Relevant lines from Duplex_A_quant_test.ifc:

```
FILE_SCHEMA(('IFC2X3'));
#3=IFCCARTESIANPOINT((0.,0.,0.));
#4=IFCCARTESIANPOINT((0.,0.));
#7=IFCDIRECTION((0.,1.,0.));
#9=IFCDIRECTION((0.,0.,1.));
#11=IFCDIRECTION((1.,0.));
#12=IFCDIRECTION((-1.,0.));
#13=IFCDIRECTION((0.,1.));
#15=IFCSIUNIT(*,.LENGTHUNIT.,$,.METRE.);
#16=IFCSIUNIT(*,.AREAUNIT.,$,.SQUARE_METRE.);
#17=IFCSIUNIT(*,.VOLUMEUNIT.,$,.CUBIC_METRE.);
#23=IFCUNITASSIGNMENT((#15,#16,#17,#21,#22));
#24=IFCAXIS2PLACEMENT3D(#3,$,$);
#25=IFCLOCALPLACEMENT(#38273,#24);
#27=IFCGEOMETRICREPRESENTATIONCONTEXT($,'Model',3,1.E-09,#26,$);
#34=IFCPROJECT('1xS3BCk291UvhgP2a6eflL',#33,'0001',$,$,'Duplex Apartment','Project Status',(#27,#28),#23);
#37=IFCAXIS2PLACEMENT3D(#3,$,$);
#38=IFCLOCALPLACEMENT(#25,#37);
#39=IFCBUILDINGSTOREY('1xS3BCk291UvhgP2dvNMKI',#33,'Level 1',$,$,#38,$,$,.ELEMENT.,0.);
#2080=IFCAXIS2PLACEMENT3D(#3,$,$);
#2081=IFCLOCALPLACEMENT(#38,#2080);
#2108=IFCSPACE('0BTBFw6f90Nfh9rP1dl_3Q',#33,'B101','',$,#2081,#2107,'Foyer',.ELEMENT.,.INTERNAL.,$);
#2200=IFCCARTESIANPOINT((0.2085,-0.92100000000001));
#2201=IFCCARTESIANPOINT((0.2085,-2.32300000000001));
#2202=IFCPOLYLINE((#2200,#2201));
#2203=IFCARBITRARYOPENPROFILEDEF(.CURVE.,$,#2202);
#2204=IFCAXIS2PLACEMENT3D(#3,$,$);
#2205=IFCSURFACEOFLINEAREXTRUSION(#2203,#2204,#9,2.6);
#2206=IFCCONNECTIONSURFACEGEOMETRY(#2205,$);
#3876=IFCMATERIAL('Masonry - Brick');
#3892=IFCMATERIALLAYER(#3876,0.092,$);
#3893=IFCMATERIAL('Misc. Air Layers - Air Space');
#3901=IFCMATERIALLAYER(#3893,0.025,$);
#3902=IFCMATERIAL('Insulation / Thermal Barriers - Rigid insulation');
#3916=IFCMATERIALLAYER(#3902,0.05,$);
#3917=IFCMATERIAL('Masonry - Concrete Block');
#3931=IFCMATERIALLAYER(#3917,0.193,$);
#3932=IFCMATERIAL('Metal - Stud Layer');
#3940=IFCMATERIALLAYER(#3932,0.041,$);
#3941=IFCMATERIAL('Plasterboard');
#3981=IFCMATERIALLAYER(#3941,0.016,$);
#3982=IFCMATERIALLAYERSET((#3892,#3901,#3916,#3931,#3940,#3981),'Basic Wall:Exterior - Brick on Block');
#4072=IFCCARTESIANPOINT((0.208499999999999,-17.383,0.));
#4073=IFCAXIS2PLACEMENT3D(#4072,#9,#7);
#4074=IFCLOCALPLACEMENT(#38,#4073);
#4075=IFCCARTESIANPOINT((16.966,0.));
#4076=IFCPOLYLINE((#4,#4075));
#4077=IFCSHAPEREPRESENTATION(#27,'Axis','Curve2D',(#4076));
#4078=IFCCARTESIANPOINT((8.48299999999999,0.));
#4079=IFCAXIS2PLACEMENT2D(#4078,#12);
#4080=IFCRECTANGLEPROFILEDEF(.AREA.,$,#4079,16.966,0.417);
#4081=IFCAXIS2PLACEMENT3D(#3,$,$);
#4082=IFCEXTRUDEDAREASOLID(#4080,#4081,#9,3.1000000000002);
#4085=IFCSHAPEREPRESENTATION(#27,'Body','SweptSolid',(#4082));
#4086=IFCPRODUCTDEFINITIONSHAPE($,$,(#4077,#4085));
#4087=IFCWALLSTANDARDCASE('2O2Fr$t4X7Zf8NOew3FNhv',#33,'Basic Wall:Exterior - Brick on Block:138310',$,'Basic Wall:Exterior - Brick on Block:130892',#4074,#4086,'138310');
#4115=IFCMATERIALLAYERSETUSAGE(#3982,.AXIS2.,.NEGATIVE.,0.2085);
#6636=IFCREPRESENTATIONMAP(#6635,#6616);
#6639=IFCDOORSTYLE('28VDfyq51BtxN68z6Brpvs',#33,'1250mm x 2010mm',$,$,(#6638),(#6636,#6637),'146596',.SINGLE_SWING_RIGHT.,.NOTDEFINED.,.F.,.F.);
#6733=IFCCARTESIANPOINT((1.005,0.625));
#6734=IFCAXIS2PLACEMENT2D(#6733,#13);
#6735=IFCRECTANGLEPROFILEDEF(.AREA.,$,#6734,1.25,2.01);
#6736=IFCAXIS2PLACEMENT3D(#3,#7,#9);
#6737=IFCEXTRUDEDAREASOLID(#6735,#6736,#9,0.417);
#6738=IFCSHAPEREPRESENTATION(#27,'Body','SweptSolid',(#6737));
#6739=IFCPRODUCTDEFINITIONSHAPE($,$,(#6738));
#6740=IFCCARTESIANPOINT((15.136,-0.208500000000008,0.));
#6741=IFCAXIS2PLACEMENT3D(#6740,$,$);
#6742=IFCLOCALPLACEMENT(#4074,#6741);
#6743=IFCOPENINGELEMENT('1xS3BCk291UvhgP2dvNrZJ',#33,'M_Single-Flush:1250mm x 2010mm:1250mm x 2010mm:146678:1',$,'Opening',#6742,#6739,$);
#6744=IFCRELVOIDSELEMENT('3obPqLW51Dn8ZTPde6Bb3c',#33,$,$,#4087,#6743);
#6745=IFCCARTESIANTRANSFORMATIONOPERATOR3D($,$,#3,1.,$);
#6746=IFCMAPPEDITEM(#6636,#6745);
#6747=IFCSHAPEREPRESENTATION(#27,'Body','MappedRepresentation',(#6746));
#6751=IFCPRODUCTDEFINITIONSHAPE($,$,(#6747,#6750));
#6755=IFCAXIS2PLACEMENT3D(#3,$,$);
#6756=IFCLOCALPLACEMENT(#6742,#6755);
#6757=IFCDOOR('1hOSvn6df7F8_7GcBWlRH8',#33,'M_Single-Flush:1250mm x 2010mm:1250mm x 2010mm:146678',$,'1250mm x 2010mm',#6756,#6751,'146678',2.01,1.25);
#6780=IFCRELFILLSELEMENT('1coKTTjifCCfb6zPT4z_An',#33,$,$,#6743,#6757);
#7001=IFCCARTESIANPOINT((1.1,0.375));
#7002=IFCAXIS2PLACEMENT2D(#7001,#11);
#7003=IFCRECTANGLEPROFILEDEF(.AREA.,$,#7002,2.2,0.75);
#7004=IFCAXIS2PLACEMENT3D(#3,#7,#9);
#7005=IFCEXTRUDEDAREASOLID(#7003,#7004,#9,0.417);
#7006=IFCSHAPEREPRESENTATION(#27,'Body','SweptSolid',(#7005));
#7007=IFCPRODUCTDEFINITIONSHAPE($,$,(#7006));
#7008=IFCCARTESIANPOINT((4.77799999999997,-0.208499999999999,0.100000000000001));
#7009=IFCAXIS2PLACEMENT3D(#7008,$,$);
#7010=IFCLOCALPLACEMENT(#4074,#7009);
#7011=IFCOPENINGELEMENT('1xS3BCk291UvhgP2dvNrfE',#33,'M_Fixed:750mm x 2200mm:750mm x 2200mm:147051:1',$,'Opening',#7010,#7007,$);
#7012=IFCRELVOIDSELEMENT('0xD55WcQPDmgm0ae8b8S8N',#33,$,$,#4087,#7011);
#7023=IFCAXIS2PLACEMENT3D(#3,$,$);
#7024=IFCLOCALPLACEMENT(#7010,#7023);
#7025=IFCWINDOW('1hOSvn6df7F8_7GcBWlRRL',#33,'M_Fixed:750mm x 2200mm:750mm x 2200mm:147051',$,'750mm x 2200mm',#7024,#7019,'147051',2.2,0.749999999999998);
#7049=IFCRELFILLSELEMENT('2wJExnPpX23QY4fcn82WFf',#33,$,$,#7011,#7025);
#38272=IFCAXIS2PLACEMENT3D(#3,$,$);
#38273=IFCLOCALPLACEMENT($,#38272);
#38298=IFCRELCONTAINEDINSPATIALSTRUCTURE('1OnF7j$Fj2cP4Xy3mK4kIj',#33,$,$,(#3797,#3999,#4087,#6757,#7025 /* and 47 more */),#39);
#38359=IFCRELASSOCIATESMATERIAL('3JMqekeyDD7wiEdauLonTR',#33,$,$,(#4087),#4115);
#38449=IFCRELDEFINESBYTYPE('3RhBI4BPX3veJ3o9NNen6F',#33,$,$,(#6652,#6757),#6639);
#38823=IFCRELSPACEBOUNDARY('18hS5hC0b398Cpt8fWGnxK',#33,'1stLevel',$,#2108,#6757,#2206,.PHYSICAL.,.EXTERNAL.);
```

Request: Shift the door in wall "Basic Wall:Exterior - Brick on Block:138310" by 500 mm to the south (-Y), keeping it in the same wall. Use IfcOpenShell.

```python
import numpy as np
import ifcopenshell
import ifcopenshell.api.geometry
import ifcopenshell.util.placement
import ifcopenshell.util.unit

model = ifcopenshell.open("Duplex_A_quant_test.ifc")
unit_scale = ifcopenshell.util.unit.calculate_unit_scale(model)

door = model.by_id(6757)
opening = door.FillsVoids[0].RelatingOpeningElement
wall = opening.VoidsElements[0].RelatingBuildingElement

wall_matrix = ifcopenshell.util.placement.get_local_placement(wall.ObjectPlacement)
shift = wall_matrix[:3, 0] * -0.5 / unit_scale
before = ifcopenshell.util.placement.get_local_placement(door.ObjectPlacement)[:3, 3].copy()

# The door is placed relative to its opening, so it follows when the opening moves.
matrix = ifcopenshell.util.placement.get_local_placement(opening.ObjectPlacement)
matrix[:3, 3] += shift
ifcopenshell.api.geometry.edit_object_placement(
    model, product=opening, matrix=matrix, is_si=False, should_transform_children=True
)

# Space boundary surfaces are stored in each space's coordinates; move them too.
for rel in door.ProvidesBoundaries:
    if not rel.ConnectionGeometry:
        continue
    surface = rel.ConnectionGeometry.SurfaceOnRelatingElement
    space_matrix = ifcopenshell.util.placement.get_local_placement(rel.RelatingSpace.ObjectPlacement)
    point = np.array(surface.Position.Location.Coordinates) + space_matrix[:3, :3].T @ shift
    surface.Position = model.createIfcAxis2Placement3D(
        model.createIfcCartesianPoint(point.tolist()), surface.Position.Axis, surface.Position.RefDirection
    )

after = ifcopenshell.util.placement.get_local_placement(door.ObjectPlacement)[:3, 3]
print("door moved by", (after - before).round(3) + 0.0)

model.write("Duplex_A_quant_test-out.ifc")
```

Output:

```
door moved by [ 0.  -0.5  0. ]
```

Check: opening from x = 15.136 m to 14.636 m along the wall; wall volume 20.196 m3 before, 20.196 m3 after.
